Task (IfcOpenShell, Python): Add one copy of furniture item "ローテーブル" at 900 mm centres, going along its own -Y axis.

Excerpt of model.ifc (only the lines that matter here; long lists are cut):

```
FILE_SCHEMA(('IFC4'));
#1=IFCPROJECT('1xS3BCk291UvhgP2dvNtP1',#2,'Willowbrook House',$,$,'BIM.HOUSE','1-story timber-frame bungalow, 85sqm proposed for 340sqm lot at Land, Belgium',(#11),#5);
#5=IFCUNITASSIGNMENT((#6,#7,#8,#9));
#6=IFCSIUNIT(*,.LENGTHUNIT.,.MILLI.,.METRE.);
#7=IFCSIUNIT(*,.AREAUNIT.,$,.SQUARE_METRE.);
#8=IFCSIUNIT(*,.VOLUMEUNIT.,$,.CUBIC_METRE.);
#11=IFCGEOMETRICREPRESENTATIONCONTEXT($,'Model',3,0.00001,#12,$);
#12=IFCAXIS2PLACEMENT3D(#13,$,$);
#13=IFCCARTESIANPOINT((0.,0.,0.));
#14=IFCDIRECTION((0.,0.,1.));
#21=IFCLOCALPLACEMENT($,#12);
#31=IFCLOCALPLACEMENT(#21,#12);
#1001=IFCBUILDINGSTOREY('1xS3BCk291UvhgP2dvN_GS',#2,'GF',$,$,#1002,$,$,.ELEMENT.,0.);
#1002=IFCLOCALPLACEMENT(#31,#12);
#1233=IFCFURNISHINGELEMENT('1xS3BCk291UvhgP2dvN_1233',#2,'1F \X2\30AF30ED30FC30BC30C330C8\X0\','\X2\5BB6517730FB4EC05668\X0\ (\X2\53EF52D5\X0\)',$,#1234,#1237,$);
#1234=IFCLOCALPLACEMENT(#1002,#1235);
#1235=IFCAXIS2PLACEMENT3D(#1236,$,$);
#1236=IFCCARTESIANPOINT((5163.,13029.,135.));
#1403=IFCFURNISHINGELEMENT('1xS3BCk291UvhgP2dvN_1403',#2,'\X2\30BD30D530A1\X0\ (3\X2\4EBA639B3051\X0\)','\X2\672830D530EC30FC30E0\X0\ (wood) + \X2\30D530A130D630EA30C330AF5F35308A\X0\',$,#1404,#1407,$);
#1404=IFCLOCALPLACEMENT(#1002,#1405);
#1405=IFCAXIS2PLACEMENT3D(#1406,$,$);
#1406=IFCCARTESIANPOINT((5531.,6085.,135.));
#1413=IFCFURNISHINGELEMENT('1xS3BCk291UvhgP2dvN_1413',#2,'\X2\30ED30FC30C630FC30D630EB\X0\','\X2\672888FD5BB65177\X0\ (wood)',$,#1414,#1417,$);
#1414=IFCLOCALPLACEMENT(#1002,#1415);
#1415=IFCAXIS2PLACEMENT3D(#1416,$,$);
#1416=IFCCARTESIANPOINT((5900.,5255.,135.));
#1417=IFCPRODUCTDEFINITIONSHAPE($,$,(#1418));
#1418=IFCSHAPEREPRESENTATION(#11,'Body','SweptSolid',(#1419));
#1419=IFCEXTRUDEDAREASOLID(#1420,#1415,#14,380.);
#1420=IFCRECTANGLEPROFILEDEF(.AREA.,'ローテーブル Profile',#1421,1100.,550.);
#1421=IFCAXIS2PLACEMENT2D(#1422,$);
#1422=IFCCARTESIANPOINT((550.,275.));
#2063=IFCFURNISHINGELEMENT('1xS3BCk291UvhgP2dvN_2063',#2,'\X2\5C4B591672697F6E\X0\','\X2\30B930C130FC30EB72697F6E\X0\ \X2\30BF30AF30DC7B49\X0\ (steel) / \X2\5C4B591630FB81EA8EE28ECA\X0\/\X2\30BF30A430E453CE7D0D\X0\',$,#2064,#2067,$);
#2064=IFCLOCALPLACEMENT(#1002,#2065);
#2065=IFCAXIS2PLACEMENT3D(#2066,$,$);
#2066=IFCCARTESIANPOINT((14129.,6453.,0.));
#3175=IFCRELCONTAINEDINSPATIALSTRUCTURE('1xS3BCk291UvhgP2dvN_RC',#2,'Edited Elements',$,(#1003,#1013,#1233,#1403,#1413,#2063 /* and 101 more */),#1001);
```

```python
import ifcopenshell
import ifcopenshell.api.geometry
import ifcopenshell.api.root
import ifcopenshell.util.element
import ifcopenshell.util.placement
import ifcopenshell.util.unit

model = ifcopenshell.open("model.ifc")
unit_scale = ifcopenshell.util.unit.calculate_unit_scale(model)


def reuse_history(source, copy):
    """copy_class also copies each property set's owner history, people and application; keep the originals."""
    for rel in copy.IsDefinedBy:
        if rel.is_a("IfcRelDefinesByProperties") and (history := rel.RelatingPropertyDefinition.OwnerHistory):
            rel.RelatingPropertyDefinition.OwnerHistory = source.OwnerHistory
            ifcopenshell.util.element.remove_deep2(model, history)


source = model.by_id(1413)
base = ifcopenshell.util.placement.get_local_placement(source.ObjectPlacement)
step = -base[:3, 1] * 0.9 / unit_scale

for i in range(1, 2):
    copy = ifcopenshell.api.root.copy_class(model, product=source)
    copy.Representation = ifcopenshell.util.element.copy_deep(
        model, source.Representation, exclude=["IfcGeometricRepresentationContext", "IfcRepresentationMap"]
    )
    reuse_history(source, copy)
    matrix = base.copy()
    matrix[:3, 3] += i * step
    print("added at", matrix[:3, 3].round(3) + 0.0)
    ifcopenshell.api.geometry.edit_object_placement(model, product=copy, matrix=matrix, is_si=False)

model.write("model_edited.ifc")
```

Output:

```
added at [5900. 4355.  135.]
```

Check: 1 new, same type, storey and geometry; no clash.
